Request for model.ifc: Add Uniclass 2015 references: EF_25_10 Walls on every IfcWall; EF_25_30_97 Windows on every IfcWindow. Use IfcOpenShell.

First a look at what the model holds.

```python
import ifcopenshell

model = ifcopenshell.open("model.ifc")
print(model.schema)
print("classifications:", [c.Name for c in model.by_type("IfcClassification")])
for ifc_class in ("IfcDoor", "IfcRoof", "IfcStair", "IfcWall", "IfcWindow"):
    print(ifc_class, len(model.by_type(ifc_class)))
```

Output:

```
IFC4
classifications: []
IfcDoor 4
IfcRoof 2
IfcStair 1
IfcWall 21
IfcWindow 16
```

```python
import ifcopenshell
import ifcopenshell.api.classification

model = ifcopenshell.open("model.ifc")

system = ifcopenshell.api.classification.add_classification(model, classification="Uniclass 2015")

codes = {
    "IfcWall": ("EF_25_10", "Walls"),
    "IfcWindow": ("EF_25_30_97", "Windows"),
}
for ifc_class, (code, name) in codes.items():
    products = model.by_type(ifc_class)
    ifcopenshell.api.classification.add_reference(
        model, products=products, classification=system, identification=code, name=name
    )
    print(code, len(products))

model.write("model_v2.ifc")
```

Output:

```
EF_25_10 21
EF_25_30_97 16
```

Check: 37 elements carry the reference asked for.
